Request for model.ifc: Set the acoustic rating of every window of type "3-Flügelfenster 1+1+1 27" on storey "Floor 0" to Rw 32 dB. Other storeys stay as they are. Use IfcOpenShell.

First a look at what the model holds.

```python
import ifcopenshell
import ifcopenshell.util.element

model = ifcopenshell.open("model.ifc")
print(model.schema)
storey = next(s for s in model.by_type("IfcBuildingStorey") if s.Name == "Floor 0")
windows = [e for e in ifcopenshell.util.element.get_decomposition(storey) if e.is_a("IfcWindow")]
seen = {}
for e in windows:
    element_type = ifcopenshell.util.element.get_type(e)
    key = (element_type.Name if element_type != e and element_type else None, ifcopenshell.util.element.get_pset(e, "Pset_WindowCommon", "AcousticRating"))
    seen[key] = seen.get(key, 0) + 1
for (name, value), count in sorted(seen.items(), key=str):
    print(count, "x", name, "|", value)
```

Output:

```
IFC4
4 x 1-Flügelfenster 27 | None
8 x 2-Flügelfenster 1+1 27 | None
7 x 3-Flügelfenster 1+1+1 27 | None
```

```python
import ifcopenshell
import ifcopenshell.api.pset
import ifcopenshell.util.element

model = ifcopenshell.open("model.ifc")

storey = next(s for s in model.by_type("IfcBuildingStorey") if s.Name == "Floor 0")
windows = [e for e in ifcopenshell.util.element.get_decomposition(storey) if e.is_a("IfcWindow")]

count = 0
for e in windows:
    element_type = ifcopenshell.util.element.get_type(e)
    if element_type in (None, e) or element_type.Name != "3-Flügelfenster 1+1+1 27":
        continue
    # add_pset returns the element's existing set when there is one.
    pset = ifcopenshell.api.pset.add_pset(model, product=e, name="Pset_WindowCommon")
    ifcopenshell.api.pset.edit_pset(model, pset=pset, properties={"AcousticRating": "Rw 32 dB"})
    count += 1

print(count, "windows updated")

model.write("model_rev.ifc")
```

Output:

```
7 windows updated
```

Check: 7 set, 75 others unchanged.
